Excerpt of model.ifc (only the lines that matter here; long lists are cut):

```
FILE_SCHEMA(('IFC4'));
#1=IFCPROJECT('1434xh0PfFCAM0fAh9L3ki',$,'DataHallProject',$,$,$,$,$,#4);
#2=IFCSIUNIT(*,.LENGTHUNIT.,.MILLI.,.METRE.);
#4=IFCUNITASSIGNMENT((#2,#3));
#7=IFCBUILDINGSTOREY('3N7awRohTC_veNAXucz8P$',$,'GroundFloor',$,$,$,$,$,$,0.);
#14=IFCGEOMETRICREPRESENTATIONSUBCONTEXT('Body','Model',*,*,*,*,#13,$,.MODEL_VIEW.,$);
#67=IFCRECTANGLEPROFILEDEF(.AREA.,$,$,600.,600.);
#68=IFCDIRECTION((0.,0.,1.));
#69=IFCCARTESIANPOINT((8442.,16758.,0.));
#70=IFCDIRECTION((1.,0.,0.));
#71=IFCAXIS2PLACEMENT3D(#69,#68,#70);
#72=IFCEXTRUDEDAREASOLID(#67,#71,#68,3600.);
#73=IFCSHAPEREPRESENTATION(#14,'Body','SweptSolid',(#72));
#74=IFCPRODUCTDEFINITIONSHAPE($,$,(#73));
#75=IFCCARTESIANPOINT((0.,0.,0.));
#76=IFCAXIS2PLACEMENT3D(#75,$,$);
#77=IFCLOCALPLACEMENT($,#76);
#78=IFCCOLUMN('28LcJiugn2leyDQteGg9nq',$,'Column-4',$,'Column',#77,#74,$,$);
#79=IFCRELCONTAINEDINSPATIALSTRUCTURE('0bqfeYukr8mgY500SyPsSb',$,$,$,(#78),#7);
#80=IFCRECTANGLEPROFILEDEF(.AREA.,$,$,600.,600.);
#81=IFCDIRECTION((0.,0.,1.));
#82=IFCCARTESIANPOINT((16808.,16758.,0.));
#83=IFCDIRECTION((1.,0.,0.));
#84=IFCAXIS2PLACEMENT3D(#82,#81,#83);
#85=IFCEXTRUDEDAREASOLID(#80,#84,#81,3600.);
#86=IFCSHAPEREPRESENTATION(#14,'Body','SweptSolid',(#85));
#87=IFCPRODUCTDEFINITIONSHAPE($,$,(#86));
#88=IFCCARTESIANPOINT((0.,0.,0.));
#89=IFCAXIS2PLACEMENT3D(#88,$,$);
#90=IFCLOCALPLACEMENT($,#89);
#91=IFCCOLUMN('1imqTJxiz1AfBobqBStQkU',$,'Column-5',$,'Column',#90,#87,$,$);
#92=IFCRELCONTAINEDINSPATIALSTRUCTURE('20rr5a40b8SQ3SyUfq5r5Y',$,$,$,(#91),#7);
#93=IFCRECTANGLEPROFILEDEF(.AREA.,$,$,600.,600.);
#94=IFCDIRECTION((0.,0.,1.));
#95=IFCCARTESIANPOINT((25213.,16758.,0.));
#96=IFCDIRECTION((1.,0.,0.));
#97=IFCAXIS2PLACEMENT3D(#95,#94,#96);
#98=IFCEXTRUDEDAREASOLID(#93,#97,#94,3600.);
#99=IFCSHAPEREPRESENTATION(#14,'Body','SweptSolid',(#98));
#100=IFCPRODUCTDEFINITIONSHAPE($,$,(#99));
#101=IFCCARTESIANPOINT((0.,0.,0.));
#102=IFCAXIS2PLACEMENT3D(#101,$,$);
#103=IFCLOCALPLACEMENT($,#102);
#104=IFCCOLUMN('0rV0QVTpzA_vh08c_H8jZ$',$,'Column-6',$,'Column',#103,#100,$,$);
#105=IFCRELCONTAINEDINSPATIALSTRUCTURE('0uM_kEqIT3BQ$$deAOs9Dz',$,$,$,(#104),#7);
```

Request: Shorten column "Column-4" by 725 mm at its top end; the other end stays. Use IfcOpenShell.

```python
import ifcopenshell
import ifcopenshell.util.representation
import ifcopenshell.util.unit

model = ifcopenshell.open("model.ifc")
unit_scale = ifcopenshell.util.unit.calculate_unit_scale(model)

member = model.by_guid("28LcJiugn2leyDQteGg9nq")
change = -0.725 / unit_scale

# The extrusion runs towards the end named, so only its depth changes.
body = ifcopenshell.util.representation.get_representation(member, "Model", "Body")
solid = body.Items[0]
old_length = solid.Depth
solid.Depth += change

print(f"length {old_length:g} -> {solid.Depth:g}")

model.write("model_v2.ifc")
```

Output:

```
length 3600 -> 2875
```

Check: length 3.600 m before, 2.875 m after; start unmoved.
